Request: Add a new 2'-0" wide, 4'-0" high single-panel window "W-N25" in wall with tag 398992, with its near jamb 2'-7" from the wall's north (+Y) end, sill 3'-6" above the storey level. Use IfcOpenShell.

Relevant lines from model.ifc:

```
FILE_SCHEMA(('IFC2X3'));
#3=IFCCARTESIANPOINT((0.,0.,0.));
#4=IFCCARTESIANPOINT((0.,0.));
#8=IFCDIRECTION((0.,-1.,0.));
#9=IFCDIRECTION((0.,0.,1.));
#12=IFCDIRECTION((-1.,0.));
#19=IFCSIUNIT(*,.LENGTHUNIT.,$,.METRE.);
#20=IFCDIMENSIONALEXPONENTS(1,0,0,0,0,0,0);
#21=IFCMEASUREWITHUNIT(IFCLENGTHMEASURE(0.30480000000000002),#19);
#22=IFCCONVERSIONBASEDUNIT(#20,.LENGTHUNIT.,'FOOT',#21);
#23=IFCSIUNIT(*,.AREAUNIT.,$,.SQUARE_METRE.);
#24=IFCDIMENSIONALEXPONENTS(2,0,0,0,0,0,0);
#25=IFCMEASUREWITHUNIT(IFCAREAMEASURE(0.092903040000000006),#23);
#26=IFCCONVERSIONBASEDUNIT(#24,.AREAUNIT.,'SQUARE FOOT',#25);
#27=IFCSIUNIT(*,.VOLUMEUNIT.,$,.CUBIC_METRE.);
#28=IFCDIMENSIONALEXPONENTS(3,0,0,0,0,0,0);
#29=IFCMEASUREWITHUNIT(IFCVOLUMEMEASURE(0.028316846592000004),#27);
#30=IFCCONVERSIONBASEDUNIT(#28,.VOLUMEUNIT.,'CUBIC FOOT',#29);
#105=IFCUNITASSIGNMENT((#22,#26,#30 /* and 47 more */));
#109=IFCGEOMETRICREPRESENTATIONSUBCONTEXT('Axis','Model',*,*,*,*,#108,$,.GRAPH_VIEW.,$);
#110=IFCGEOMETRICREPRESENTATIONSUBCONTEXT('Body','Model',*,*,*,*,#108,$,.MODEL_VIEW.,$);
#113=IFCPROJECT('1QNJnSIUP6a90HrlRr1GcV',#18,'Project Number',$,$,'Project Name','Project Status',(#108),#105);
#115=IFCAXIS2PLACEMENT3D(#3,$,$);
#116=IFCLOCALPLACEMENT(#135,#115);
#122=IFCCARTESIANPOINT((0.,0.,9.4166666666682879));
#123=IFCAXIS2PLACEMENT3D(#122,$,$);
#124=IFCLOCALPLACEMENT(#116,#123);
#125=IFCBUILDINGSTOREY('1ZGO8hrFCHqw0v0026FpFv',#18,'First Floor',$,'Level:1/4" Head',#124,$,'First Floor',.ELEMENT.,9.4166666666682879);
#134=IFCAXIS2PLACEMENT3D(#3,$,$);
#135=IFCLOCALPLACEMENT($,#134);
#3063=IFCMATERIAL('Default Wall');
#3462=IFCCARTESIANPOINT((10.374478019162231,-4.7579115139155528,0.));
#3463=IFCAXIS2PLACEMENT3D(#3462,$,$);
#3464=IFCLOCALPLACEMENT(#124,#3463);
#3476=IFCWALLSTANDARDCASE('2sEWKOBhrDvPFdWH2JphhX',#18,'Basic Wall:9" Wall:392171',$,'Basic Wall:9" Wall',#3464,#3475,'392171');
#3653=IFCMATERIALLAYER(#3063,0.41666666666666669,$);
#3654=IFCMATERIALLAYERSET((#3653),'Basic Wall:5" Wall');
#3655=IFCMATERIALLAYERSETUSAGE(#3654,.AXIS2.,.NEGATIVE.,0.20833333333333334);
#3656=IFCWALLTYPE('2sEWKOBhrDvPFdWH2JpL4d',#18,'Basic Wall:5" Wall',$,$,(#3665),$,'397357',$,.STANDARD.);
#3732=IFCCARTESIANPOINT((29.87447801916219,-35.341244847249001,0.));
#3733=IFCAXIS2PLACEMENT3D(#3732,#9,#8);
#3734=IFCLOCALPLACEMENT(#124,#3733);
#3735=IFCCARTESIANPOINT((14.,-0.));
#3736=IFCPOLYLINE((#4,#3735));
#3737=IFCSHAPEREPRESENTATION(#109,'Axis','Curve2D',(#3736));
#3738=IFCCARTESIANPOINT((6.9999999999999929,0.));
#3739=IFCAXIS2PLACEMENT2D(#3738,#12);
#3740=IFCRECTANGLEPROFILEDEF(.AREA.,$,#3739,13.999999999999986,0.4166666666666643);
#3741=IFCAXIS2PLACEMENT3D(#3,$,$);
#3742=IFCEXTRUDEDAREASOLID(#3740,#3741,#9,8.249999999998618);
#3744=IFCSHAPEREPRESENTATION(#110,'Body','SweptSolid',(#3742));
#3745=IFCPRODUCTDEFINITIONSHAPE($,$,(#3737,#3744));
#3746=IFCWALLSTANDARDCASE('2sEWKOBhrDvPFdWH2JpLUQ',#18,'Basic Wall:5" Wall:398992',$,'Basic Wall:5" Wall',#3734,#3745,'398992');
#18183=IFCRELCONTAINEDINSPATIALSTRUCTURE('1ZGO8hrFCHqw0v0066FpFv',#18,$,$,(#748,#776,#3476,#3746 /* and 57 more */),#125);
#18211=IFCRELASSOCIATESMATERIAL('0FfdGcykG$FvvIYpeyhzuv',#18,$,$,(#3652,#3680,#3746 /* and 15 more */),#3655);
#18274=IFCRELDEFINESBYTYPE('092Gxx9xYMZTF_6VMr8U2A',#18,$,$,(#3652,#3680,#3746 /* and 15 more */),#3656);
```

```python
import numpy as np
import ifcopenshell
import ifcopenshell.api.feature
import ifcopenshell.api.geometry
import ifcopenshell.api.root
import ifcopenshell.api.spatial
import ifcopenshell.api.type
import ifcopenshell.geom
import ifcopenshell.util.element
import ifcopenshell.util.placement
import ifcopenshell.util.representation
import ifcopenshell.util.shape
import ifcopenshell.util.unit

model = ifcopenshell.open("model.ifc")
unit_scale = ifcopenshell.util.unit.calculate_unit_scale(model)
settings = ifcopenshell.geom.settings()


def volume(element):
    """Net volume in cubic metres, openings subtracted."""
    shape = ifcopenshell.geom.create_shape(settings, element)
    return ifcopenshell.util.shape.get_volume(shape.geometry)


wall = model.by_guid("2sEWKOBhrDvPFdWH2JpLUQ")
storey = ifcopenshell.util.element.get_container(wall, ifc_class="IfcBuildingStorey")
context = ifcopenshell.util.representation.get_context(model, "Model", "Body", "MODEL_VIEW")
before = volume(wall)

width, height, from_end, sill = 0.6096, 1.2192, 0.7874, 1.0668  # metres

# The wall runs along its own X axis, and the end named is its -X end.
wall_shape = ifcopenshell.geom.create_shape(settings, wall)
x, y, z = ifcopenshell.util.shape.get_vertices(wall_shape.geometry).T
start = x.min() + from_end
face, thickness = float(y.min()), float(y.max() - y.min())
wall_matrix = ifcopenshell.util.placement.get_local_placement(wall.ObjectPlacement)
level = ifcopenshell.util.placement.get_local_placement(storey.ObjectPlacement)[2, 3]


def in_wall(x, y):
    """Placement at x, y metres in the wall's axes, at sill height."""
    matrix = wall_matrix.copy()
    matrix[:, 3] = wall_matrix @ np.array([x / unit_scale, y / unit_scale, 0.0, 1.0])
    matrix[2, 3] = level + sill / unit_scale
    return matrix


# Opening: a box that overshoots both wall faces by 50 mm.
opening = ifcopenshell.api.root.create_entity(model, ifc_class="IfcOpeningElement")
box = ifcopenshell.api.geometry.add_wall_representation(
    model, context=context, length=width, height=height, thickness=thickness + 0.1
)
ifcopenshell.api.geometry.assign_representation(model, product=opening, representation=box)
ifcopenshell.api.geometry.edit_object_placement(model, product=opening, matrix=in_wall(start, face - 0.05), is_si=False)
ifcopenshell.api.feature.add_feature(model, feature=opening, element=wall)

window = ifcopenshell.api.root.create_entity(model, ifc_class="IfcWindow", name="W-N25")
window.OverallWidth, window.OverallHeight = width / unit_scale, height / unit_scale
body = ifcopenshell.api.geometry.add_window_representation(
    model,
    context=context,
    overall_width=window.OverallWidth,
    overall_height=window.OverallHeight,
    partition_type="SINGLE_PANEL",
)
ifcopenshell.api.geometry.assign_representation(model, product=window, representation=body)
ifcopenshell.api.spatial.assign_container(model, products=[window], relating_structure=storey)
fills = ifcopenshell.api.feature.add_filling(model, opening=opening, element=window)
fills.OwnerHistory = window.OwnerHistory  # required in IFC2X3

# IFC2X3 keeps the operation on the window style.
style = ifcopenshell.api.root.create_entity(model, ifc_class="IfcWindowStyle", name="W-N25")
style.OperationType, style.ConstructionType = "SINGLE_PANEL", "NOTDEFINED"
style.ParameterTakesPrecedence = style.Sizeable = False
ifcopenshell.api.type.assign_type(model, related_objects=[window], relating_type=style)

# Centre the window in the wall's thickness.
ifcopenshell.api.geometry.edit_object_placement(model, product=window, matrix=in_wall(start, face), is_si=False)
window_shape = ifcopenshell.geom.create_shape(settings, window)
depth = ifcopenshell.util.shape.get_vertices(window_shape.geometry)[:, 1]
offset = face + thickness / 2 - (depth.min() + depth.max()) / 2
ifcopenshell.api.geometry.edit_object_placement(model, product=window, matrix=in_wall(start, offset), is_si=False)

after = volume(wall)

print(f"wall volume {before:.3f} -> {after:.3f} m3")

model.write("model-out.ifc")
```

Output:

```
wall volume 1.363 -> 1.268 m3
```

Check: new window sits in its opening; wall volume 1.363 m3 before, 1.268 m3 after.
